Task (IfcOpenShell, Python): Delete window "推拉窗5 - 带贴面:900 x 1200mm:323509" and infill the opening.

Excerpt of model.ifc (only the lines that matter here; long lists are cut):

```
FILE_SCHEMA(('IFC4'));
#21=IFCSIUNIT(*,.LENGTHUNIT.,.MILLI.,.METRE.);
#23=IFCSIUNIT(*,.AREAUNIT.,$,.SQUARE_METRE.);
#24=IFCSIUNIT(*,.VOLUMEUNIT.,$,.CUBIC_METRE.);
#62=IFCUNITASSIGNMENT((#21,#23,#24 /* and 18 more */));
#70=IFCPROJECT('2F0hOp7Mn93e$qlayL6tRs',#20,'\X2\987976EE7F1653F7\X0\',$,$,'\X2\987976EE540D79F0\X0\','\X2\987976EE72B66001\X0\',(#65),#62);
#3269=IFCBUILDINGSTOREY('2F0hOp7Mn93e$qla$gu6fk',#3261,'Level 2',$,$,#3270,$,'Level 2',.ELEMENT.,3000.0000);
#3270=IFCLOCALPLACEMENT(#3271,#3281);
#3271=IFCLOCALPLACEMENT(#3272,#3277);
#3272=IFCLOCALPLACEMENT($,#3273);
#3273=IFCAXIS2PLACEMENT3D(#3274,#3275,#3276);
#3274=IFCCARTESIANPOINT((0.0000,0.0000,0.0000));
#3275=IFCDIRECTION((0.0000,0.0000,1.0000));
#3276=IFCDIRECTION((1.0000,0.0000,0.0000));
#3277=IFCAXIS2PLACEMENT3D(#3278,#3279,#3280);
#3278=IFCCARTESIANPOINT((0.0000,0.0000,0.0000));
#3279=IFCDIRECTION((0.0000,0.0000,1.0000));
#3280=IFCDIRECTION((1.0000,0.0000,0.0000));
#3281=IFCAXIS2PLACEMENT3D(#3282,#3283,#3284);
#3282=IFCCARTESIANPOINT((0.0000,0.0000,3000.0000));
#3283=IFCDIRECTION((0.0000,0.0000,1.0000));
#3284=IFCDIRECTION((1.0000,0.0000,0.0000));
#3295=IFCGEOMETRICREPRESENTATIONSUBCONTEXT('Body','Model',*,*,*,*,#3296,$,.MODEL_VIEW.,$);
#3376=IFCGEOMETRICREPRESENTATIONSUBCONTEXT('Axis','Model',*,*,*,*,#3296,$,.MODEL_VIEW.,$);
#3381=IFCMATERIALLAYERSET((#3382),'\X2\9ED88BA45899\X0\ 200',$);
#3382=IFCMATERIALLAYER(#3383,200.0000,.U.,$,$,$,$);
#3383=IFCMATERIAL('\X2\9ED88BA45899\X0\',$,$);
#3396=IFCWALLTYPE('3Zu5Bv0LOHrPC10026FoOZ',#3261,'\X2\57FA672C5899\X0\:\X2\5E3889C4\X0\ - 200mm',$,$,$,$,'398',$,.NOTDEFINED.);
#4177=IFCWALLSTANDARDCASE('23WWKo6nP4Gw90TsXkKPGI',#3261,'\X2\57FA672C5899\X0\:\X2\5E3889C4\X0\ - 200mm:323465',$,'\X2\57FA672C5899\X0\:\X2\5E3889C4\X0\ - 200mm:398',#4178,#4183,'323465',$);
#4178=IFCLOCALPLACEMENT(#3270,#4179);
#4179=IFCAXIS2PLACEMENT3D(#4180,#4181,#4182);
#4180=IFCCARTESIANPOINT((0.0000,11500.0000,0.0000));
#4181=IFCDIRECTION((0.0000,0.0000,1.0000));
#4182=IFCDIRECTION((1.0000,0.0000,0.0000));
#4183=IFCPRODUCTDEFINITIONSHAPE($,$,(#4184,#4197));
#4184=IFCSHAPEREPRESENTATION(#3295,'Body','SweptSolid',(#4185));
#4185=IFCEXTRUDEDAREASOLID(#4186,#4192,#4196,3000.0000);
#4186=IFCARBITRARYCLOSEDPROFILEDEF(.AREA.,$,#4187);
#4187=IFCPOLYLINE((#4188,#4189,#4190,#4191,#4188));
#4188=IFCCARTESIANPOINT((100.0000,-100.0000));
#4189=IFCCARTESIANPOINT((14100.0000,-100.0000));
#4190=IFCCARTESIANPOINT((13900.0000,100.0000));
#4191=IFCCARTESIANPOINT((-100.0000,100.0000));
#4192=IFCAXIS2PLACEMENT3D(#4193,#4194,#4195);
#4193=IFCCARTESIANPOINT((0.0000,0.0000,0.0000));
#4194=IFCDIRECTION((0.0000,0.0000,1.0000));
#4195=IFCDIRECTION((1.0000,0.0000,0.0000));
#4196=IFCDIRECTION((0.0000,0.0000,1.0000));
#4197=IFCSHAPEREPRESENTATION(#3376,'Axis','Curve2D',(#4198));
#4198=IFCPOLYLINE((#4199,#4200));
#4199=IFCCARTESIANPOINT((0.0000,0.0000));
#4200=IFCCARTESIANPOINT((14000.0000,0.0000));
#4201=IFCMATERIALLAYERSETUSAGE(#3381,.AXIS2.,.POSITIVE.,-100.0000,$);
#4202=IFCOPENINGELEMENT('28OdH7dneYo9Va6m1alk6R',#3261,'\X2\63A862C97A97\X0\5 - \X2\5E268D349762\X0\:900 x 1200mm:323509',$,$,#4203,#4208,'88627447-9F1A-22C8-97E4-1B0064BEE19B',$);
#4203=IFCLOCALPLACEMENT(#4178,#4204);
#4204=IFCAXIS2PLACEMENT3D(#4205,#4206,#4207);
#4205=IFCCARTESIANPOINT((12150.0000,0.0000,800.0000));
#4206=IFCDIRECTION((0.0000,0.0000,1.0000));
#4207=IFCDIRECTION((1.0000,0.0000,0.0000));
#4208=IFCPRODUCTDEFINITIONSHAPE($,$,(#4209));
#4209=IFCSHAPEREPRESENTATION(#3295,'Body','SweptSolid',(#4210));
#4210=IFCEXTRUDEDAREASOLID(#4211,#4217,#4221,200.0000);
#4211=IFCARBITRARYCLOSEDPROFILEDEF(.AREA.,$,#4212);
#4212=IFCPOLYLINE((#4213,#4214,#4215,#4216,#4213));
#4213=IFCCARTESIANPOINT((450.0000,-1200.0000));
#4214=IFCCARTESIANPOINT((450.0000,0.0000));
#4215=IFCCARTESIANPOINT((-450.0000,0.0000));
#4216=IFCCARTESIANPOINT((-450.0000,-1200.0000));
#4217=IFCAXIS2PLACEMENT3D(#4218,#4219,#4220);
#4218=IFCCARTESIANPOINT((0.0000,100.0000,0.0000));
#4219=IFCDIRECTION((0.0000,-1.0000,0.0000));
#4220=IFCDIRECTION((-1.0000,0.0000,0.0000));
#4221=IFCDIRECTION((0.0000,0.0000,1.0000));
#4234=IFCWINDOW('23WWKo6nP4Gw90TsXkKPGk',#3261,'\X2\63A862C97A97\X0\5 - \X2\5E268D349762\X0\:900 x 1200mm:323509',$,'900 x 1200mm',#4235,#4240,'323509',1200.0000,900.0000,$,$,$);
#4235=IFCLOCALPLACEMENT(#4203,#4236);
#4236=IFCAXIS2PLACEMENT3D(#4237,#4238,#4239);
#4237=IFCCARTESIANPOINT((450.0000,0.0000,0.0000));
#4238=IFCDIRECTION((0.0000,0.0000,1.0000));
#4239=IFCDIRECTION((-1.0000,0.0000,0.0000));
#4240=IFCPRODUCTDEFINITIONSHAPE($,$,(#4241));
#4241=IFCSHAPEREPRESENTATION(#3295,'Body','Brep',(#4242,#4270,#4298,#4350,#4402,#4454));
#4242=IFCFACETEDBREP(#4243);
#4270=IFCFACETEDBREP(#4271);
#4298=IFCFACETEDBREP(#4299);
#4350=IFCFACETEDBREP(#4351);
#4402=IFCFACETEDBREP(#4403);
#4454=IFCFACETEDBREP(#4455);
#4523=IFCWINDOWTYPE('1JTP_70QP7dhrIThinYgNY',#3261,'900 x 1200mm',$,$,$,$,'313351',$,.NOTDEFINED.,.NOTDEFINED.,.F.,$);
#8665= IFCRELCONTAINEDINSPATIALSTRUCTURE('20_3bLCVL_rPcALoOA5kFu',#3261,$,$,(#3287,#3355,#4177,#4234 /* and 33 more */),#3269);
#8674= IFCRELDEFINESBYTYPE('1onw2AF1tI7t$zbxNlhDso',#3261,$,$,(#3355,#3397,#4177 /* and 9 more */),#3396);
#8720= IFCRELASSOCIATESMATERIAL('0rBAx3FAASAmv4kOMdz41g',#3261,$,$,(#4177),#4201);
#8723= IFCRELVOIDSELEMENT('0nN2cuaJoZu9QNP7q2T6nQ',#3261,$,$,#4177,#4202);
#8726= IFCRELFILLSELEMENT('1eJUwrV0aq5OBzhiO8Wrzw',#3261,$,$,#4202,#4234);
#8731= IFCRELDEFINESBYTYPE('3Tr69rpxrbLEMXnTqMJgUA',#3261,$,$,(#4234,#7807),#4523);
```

```python
import ifcopenshell
import ifcopenshell.api.feature
import ifcopenshell.api.root
import ifcopenshell.geom
import ifcopenshell.util.shape

model = ifcopenshell.open("model.ifc")
settings = ifcopenshell.geom.settings()


def volume(element):
    """Net volume in cubic metres, openings subtracted."""
    shape = ifcopenshell.geom.create_shape(settings, element)
    return ifcopenshell.util.shape.get_volume(shape.geometry)


window = model.by_id(4234)
opening = window.FillsVoids[0].RelatingOpeningElement
wall = opening.VoidsElements[0].RelatingBuildingElement
before = volume(wall)

ifcopenshell.api.root.remove_product(model, product=window)
ifcopenshell.api.feature.remove_feature(model, feature=opening)

after = volume(wall)

print(f"wall volume {before:.3f} -> {after:.3f} m3")

model.write("model-out.ifc")
```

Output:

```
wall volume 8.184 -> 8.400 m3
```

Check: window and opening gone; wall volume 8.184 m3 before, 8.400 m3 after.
